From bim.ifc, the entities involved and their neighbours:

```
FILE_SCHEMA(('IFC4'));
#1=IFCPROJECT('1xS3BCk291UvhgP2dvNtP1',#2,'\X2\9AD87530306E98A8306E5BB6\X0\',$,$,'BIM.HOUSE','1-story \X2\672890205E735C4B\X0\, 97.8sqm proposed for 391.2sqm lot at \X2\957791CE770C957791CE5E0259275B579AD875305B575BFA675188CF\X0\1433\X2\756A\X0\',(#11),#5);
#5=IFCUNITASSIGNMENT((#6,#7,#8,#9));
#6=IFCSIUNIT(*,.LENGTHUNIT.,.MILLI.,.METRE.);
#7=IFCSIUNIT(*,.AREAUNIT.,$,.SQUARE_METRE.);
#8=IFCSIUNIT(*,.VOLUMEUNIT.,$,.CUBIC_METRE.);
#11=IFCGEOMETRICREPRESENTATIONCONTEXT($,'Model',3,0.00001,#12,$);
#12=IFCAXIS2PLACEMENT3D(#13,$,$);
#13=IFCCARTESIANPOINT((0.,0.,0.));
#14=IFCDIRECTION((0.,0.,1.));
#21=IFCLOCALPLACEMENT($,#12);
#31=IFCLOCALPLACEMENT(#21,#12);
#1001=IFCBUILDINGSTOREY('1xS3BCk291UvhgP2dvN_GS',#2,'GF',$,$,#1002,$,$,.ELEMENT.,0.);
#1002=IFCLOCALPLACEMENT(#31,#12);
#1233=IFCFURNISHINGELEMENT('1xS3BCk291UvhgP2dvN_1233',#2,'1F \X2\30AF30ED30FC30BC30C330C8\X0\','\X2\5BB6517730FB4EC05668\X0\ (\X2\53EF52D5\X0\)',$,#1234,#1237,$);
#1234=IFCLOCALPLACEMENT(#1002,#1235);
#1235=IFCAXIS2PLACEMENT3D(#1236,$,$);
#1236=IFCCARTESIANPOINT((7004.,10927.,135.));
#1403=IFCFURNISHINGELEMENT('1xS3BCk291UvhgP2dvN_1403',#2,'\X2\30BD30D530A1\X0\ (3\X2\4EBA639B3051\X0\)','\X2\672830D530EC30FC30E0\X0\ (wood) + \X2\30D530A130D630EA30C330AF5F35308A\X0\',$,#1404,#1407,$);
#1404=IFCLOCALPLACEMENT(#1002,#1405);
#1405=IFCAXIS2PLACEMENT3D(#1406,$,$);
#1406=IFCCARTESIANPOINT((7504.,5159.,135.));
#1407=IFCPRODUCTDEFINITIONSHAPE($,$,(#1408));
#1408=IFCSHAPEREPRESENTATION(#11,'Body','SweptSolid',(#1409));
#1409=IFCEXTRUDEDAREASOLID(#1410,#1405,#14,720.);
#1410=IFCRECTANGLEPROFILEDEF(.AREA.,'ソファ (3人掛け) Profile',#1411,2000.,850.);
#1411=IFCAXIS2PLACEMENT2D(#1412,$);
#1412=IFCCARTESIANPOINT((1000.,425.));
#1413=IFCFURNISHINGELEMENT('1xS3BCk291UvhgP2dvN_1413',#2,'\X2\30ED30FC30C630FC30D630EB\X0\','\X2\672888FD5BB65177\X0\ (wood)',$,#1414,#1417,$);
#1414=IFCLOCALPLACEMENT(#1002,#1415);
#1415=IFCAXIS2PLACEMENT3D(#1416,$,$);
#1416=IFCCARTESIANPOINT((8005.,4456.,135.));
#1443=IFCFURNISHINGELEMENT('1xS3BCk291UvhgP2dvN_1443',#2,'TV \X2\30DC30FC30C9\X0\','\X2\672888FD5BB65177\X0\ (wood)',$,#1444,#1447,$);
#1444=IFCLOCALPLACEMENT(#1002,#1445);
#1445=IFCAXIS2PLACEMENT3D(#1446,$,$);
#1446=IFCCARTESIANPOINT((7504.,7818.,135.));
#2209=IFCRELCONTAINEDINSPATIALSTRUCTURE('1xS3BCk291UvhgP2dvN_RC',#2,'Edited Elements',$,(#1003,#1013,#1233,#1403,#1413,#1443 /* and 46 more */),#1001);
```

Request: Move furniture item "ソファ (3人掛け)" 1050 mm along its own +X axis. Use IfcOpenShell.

```python
import ifcopenshell
import ifcopenshell.api.geometry
import ifcopenshell.util.placement
import ifcopenshell.util.unit

model = ifcopenshell.open("bim.ifc")
unit_scale = ifcopenshell.util.unit.calculate_unit_scale(model)

item = model.by_guid("1xS3BCk291UvhgP2dvN_1403")
matrix = ifcopenshell.util.placement.get_local_placement(item.ObjectPlacement)
matrix[:3, 3] += matrix[:3, 0] * 1.05 / unit_scale
ifcopenshell.api.geometry.edit_object_placement(model, product=item, matrix=matrix, is_si=False)

print(ifcopenshell.util.placement.get_local_placement(item.ObjectPlacement).round(3) + 0.0)

model.write("bim_rev.ifc")
```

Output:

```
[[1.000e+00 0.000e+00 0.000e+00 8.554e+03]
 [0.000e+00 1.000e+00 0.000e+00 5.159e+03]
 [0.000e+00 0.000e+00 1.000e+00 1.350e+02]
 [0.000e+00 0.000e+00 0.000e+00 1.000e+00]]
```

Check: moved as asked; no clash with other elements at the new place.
